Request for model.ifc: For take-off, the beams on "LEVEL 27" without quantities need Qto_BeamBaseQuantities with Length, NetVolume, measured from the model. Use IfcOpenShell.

First a look at what the model holds.

```python
import ifcopenshell
import ifcopenshell.util.element
import ifcopenshell.util.unit

model = ifcopenshell.open("model.ifc")
print(model.schema)
for unit_type in ("LENGTHUNIT", "AREAUNIT", "VOLUMEUNIT"):
    print(unit_type, ifcopenshell.util.unit.calculate_unit_scale(model, unit_type))
storey = next(s for s in model.by_type("IfcBuildingStorey") if s.Name == "LEVEL 27")
beams = [e for e in ifcopenshell.util.element.get_decomposition(storey) if e.is_a("IfcBeam")]
for e in sorted(beams, key=lambda e: e.id()):
    print(e.id(), e.is_a(), e.Name, list(ifcopenshell.util.element.get_psets(e, qtos_only=True)), sep=" | ")
```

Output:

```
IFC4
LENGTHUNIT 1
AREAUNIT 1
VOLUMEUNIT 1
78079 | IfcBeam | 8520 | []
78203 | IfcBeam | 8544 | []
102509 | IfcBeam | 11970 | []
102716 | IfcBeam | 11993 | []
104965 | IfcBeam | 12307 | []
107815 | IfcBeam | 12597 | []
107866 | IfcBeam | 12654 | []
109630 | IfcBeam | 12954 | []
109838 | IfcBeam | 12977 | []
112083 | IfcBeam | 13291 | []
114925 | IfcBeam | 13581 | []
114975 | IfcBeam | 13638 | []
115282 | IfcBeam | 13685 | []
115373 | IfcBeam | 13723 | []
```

```python
import ifcopenshell
import ifcopenshell.api.pset
import ifcopenshell.geom
import ifcopenshell.util.element
import ifcopenshell.util.shape
import ifcopenshell.util.unit

model = ifcopenshell.open("model.ifc")
unit_scale = ifcopenshell.util.unit.calculate_unit_scale(model)
volume_scale = ifcopenshell.util.unit.calculate_unit_scale(model, "VOLUMEUNIT")
settings = ifcopenshell.geom.settings()

storey = next(s for s in model.by_type("IfcBuildingStorey") if s.Name == "LEVEL 27")
beams = [e for e in ifcopenshell.util.element.get_decomposition(storey) if e.is_a("IfcBeam")]

for e in sorted(beams, key=lambda e: e.id()):
    if ifcopenshell.util.element.get_psets(e, qtos_only=True, should_inherit=False):
        continue
    # Geometry comes back in metres, in the element's own axes.
    shape = ifcopenshell.geom.create_shape(settings, e)
    values = {
        "Length": ifcopenshell.util.shape.get_max_xyz(shape.geometry) / unit_scale,
        "NetVolume": ifcopenshell.util.shape.get_volume(shape.geometry) / volume_scale,
    }
    qto = ifcopenshell.api.pset.add_qto(model, product=e, name="Qto_BeamBaseQuantities")
    ifcopenshell.api.pset.edit_qto(model, qto=qto, properties=values)
    print(e.id(), {k: round(v, 3) for k, v in values.items()})

model.write("model_updated.ifc")
```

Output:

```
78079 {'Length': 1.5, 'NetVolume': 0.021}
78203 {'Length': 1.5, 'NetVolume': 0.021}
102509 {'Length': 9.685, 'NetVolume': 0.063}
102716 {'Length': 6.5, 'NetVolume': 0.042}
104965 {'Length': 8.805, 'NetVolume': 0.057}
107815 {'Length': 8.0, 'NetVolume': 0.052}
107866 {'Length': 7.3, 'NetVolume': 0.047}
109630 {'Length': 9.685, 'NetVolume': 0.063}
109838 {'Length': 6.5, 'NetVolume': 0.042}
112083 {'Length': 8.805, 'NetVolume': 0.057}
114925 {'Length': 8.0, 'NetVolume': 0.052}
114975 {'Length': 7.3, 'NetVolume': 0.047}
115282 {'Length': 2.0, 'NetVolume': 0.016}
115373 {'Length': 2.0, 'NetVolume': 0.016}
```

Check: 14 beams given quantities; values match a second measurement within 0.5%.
